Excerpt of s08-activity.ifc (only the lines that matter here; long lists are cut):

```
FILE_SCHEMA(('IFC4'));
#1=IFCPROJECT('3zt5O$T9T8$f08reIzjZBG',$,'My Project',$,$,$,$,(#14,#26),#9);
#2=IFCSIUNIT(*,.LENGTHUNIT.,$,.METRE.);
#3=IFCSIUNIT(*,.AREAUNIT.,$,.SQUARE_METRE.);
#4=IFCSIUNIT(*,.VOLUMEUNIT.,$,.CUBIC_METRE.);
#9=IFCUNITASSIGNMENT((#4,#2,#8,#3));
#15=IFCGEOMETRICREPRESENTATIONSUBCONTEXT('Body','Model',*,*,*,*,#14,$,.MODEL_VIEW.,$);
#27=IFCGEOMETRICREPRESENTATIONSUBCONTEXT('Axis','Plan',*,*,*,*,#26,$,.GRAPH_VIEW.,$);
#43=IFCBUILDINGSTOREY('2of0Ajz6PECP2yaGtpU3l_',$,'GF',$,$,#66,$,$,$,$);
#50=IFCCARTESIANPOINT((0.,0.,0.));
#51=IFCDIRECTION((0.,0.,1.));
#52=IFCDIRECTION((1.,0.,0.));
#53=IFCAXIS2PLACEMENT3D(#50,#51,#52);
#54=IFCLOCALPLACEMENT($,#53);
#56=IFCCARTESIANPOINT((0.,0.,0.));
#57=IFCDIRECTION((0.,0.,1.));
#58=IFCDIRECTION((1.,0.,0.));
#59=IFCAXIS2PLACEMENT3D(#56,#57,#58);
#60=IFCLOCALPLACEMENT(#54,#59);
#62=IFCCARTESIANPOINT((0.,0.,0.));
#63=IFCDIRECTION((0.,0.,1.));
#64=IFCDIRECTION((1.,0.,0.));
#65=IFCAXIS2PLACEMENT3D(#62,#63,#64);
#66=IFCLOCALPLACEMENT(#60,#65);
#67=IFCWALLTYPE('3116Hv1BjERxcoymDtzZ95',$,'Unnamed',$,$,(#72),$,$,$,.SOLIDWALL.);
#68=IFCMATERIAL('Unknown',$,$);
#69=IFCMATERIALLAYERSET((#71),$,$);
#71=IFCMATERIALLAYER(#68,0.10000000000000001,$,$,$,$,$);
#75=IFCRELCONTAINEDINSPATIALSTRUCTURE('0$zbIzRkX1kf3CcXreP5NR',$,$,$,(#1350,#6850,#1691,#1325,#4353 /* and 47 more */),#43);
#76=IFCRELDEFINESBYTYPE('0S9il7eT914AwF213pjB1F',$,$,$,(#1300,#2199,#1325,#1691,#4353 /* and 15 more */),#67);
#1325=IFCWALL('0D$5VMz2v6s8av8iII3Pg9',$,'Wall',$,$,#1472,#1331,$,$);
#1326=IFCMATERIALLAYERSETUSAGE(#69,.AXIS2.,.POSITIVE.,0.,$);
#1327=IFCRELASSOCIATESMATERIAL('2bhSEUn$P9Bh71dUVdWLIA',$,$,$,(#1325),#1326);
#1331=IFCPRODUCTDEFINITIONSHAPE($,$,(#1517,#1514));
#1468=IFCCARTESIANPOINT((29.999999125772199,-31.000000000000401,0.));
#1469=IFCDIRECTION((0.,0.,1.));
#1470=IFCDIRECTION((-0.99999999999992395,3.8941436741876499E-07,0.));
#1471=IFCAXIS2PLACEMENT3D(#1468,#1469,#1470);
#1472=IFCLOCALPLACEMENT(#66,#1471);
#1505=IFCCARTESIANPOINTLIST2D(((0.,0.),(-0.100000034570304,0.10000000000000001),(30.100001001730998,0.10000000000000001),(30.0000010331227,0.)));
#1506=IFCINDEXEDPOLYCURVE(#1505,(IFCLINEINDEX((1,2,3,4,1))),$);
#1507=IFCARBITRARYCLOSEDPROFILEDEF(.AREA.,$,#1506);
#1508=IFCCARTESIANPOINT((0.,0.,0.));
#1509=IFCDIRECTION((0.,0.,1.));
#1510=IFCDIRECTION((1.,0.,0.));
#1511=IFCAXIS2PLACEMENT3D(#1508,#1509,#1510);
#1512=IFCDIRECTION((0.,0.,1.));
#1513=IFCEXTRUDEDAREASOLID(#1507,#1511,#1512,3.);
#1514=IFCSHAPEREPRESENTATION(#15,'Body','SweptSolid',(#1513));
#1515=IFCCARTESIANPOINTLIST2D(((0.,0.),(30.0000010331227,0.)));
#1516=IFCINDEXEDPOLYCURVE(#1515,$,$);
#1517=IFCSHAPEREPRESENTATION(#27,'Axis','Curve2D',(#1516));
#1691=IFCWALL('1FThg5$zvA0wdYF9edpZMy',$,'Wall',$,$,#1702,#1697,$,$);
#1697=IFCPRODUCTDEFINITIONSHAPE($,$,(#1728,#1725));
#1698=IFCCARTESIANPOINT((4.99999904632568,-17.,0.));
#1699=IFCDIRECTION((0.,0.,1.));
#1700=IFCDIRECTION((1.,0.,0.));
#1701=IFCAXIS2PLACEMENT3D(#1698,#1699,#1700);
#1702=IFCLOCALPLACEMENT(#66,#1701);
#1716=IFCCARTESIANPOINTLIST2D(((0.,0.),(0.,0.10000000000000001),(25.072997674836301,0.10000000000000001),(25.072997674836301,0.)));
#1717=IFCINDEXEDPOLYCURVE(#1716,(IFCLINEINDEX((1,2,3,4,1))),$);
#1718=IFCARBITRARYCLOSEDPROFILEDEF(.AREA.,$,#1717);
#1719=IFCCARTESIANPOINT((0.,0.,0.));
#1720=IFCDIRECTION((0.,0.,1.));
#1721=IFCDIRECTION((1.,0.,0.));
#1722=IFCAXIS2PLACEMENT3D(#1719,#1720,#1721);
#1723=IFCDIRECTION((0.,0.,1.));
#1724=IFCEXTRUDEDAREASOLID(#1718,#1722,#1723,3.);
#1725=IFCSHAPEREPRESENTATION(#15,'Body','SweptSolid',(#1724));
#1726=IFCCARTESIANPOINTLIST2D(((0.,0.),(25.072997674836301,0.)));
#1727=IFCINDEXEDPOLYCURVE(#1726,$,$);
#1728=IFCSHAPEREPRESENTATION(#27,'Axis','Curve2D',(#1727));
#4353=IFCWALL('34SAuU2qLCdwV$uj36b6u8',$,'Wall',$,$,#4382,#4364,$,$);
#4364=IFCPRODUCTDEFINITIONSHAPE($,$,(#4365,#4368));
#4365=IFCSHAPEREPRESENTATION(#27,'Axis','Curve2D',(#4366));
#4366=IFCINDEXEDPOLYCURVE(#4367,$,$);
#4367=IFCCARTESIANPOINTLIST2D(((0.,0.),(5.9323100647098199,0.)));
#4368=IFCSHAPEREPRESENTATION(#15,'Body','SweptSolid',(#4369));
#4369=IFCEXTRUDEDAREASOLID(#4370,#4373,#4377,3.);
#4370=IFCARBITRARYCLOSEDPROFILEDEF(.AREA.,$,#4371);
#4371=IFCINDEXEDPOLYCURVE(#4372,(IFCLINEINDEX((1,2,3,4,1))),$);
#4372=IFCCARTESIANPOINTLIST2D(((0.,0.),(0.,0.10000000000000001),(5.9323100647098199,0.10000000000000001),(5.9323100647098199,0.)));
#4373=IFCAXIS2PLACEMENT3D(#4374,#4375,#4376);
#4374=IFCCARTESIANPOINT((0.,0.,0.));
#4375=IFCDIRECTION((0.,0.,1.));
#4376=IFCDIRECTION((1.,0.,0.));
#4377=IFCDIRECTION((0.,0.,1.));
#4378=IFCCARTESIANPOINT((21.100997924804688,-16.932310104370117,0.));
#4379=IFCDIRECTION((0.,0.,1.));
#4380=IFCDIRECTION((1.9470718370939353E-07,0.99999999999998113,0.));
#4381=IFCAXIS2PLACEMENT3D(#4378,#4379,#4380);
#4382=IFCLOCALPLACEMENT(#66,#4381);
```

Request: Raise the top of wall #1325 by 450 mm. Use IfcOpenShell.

```python
import ifcopenshell
import ifcopenshell.geom
import ifcopenshell.util.representation
import ifcopenshell.util.shape

model = ifcopenshell.open("s08-activity.ifc")
settings = ifcopenshell.geom.settings()


def volume(element):
    """Net volume in cubic metres, openings subtracted."""
    shape = ifcopenshell.geom.create_shape(settings, element)
    return ifcopenshell.util.shape.get_volume(shape.geometry)


wall = model.by_guid("0D$5VMz2v6s8av8iII3Pg9")
before = volume(wall)

body = ifcopenshell.util.representation.get_representation(wall, "Model", "Body")
solid = body.Items[0]
old_height = solid.Depth
solid.Depth += 0.45
after = volume(wall)

print(f"height {old_height:g} -> {solid.Depth:g}, volume {before:.3f} -> {after:.3f} m3")

model.write("s08-activity_updated.ifc")
```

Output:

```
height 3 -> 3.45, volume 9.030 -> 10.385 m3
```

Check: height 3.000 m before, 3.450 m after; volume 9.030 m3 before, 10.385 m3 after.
